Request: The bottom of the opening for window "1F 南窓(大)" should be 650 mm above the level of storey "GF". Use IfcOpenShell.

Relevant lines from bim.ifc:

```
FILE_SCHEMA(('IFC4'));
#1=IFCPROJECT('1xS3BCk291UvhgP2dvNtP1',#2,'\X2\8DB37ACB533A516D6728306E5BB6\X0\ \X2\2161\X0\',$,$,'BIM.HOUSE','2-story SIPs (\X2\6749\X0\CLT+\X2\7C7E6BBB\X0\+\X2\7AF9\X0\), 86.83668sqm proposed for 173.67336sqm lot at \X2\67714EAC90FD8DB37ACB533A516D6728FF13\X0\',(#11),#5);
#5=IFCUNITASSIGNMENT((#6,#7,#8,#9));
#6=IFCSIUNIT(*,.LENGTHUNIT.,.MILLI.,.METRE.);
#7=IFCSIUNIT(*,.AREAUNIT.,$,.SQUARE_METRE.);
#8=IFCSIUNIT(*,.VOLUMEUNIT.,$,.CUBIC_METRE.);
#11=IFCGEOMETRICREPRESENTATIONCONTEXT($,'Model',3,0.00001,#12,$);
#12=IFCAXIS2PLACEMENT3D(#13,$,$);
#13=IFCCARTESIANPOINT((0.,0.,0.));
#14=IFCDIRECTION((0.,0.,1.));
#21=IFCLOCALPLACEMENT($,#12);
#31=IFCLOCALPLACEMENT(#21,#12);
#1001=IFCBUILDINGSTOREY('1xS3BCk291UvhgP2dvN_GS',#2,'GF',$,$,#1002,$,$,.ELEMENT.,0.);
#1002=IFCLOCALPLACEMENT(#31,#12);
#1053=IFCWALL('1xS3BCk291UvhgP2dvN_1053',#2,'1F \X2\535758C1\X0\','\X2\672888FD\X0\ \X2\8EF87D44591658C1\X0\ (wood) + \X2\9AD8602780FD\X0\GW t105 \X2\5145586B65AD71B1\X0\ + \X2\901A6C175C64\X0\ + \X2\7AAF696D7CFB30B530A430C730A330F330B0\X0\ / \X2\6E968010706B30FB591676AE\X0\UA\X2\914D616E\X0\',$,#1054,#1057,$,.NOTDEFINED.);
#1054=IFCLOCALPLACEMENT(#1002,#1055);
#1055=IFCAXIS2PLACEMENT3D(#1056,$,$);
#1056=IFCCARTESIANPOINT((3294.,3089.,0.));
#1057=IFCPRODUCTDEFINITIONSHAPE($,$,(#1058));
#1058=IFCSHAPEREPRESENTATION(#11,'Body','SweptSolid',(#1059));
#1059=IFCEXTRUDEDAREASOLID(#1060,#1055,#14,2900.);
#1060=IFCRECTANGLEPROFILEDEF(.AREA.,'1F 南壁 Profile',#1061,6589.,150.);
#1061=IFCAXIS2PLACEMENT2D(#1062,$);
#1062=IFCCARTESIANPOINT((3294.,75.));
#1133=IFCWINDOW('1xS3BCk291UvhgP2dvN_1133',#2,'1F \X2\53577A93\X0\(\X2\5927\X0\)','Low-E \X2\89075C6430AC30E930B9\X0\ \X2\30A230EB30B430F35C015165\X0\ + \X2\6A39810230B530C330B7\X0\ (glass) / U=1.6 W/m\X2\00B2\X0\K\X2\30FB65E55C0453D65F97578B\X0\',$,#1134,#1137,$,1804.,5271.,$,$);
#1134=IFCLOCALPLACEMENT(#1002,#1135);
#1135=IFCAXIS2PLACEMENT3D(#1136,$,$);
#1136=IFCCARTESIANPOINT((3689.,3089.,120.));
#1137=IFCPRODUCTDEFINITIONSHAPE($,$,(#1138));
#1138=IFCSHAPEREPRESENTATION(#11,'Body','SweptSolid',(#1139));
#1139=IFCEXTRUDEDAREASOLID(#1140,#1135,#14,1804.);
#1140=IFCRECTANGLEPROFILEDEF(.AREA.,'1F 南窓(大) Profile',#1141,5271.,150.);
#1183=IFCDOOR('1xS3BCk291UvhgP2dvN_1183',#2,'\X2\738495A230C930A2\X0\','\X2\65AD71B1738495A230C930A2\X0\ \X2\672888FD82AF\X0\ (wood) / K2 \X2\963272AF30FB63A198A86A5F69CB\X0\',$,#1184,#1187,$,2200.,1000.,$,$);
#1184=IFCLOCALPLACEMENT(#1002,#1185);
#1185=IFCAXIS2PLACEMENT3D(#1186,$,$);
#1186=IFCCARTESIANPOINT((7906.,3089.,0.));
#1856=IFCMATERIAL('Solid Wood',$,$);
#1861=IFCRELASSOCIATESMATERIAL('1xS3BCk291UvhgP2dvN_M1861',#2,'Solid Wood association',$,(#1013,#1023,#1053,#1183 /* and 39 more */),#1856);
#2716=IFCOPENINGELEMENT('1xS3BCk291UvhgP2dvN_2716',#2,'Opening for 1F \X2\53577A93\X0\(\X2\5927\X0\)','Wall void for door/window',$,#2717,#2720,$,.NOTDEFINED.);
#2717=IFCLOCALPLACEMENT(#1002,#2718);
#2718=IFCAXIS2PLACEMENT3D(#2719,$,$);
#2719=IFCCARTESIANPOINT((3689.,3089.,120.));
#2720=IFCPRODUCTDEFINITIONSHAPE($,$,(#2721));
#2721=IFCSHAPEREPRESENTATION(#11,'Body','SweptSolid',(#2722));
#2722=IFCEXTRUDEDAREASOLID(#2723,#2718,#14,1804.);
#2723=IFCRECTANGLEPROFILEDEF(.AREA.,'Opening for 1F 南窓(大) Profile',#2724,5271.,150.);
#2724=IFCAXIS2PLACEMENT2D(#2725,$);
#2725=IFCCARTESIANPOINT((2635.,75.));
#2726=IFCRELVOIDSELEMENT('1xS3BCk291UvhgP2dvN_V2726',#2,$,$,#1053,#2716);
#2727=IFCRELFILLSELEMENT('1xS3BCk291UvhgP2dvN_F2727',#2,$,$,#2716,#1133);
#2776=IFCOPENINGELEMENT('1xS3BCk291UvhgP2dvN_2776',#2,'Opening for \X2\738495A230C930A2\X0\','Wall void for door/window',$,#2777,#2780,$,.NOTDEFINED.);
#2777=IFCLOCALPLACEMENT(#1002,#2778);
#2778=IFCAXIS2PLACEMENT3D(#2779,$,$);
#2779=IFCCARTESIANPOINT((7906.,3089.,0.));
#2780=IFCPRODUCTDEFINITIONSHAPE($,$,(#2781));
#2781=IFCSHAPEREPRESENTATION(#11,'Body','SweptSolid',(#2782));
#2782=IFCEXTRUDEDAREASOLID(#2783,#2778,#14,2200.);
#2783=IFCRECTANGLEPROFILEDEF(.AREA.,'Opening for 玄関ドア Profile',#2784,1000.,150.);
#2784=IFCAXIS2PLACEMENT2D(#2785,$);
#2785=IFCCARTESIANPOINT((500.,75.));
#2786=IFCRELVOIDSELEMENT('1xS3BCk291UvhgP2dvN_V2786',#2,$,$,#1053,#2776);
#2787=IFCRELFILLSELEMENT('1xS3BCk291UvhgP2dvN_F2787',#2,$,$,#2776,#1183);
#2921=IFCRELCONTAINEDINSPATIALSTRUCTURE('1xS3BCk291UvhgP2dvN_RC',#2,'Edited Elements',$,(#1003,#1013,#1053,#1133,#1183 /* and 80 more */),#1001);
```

```python
import numpy as np
import ifcopenshell
import ifcopenshell.api.geometry
import ifcopenshell.geom
import ifcopenshell.util.element
import ifcopenshell.util.placement
import ifcopenshell.util.shape
import ifcopenshell.util.unit

model = ifcopenshell.open("bim.ifc")
unit_scale = ifcopenshell.util.unit.calculate_unit_scale(model)

window = model.by_guid("1xS3BCk291UvhgP2dvN_1133")
opening = window.FillsVoids[0].RelatingOpeningElement
storey = ifcopenshell.util.element.get_container(window, ifc_class="IfcBuildingStorey")
level = ifcopenshell.util.placement.get_local_placement(storey.ObjectPlacement)[2, 3]

# The opening's origin need not be at the sill, so measure its lowest point.
shape = ifcopenshell.geom.create_shape(ifcopenshell.geom.settings(), opening)
bottom = ifcopenshell.util.shape.get_shape_bottom_elevation(shape, shape.geometry) / unit_scale
dz = level + 0.65 / unit_scale - bottom

shift = np.array([0.0, 0.0, dz])
# The window is not placed relative to its opening, so move both.
for product in (opening, window):
    matrix = ifcopenshell.util.placement.get_local_placement(product.ObjectPlacement)
    matrix[:3, 3] += shift
    ifcopenshell.api.geometry.edit_object_placement(model, product=product, matrix=matrix, is_si=False)

print(f"moved by {dz * unit_scale:+.3f} m")

model.write("bim_v2.ifc")
```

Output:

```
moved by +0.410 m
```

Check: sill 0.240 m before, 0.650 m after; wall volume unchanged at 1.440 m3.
